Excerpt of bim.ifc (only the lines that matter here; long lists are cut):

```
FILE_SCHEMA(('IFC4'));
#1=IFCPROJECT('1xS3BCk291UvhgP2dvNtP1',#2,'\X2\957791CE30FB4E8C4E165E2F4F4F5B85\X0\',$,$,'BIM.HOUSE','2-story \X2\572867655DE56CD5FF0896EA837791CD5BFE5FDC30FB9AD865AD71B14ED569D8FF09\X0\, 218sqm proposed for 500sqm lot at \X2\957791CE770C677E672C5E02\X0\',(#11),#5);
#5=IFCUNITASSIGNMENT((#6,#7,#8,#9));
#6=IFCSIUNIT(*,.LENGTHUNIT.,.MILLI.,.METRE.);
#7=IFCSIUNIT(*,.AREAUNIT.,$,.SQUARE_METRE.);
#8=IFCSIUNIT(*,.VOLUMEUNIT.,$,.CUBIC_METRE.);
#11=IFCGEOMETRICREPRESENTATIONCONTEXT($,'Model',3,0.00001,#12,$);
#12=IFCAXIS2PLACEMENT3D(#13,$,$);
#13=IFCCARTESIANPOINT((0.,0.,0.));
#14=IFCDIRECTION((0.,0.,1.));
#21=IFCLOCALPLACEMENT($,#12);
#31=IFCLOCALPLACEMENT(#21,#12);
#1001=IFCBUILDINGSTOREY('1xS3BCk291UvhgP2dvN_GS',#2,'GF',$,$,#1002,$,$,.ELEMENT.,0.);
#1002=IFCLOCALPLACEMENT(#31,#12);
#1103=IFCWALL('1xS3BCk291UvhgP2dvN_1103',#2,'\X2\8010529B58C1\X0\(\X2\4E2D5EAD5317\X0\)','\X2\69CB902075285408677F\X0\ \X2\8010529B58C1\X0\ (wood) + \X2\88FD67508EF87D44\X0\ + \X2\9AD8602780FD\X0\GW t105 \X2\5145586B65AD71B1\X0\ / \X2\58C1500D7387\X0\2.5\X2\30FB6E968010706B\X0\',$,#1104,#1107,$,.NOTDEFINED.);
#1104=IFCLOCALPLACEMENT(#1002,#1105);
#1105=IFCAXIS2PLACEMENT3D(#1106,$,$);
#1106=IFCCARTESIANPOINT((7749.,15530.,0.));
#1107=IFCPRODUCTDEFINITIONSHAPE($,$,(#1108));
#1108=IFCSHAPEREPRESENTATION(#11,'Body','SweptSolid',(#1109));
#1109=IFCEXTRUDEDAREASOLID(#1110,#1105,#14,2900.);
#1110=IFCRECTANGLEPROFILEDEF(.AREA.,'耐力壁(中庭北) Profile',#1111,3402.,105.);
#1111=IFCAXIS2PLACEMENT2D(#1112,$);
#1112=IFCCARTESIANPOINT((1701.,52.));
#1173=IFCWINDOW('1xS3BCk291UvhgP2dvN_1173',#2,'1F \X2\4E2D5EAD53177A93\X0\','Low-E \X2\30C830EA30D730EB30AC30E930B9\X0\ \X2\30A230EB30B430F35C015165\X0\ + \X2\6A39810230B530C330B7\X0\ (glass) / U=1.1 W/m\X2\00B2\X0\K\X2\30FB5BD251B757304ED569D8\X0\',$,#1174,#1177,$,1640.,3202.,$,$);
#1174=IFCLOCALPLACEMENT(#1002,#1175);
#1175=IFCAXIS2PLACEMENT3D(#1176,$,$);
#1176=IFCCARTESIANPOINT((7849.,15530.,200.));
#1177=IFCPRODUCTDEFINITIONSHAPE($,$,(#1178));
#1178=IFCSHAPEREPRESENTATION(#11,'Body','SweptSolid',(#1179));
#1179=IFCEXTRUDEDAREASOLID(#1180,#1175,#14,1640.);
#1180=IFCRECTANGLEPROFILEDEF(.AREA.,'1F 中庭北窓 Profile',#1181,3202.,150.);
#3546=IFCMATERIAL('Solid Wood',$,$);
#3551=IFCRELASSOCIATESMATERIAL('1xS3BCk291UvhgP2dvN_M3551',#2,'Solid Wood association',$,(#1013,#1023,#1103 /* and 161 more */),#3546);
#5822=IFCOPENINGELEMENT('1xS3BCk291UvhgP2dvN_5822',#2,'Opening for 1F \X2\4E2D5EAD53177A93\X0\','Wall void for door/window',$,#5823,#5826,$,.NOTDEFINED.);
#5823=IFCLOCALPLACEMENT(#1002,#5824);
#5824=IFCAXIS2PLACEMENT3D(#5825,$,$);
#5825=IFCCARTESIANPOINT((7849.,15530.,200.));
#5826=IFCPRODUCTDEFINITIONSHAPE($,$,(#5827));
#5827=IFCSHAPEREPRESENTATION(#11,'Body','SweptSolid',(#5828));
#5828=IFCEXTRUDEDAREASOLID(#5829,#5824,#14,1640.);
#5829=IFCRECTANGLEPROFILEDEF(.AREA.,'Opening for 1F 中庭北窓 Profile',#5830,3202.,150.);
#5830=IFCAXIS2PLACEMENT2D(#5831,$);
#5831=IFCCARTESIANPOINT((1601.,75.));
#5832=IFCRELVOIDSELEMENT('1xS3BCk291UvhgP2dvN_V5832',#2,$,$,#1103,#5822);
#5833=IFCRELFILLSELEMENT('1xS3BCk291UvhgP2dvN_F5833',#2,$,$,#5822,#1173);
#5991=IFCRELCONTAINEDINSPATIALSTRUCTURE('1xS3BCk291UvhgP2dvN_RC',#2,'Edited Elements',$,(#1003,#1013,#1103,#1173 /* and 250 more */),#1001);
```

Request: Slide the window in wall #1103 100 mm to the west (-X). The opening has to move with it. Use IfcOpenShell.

```python
import ifcopenshell
import ifcopenshell.api.geometry
import ifcopenshell.util.placement
import ifcopenshell.util.unit

model = ifcopenshell.open("bim.ifc")
unit_scale = ifcopenshell.util.unit.calculate_unit_scale(model)

window = model.by_guid("1xS3BCk291UvhgP2dvN_1173")
opening = window.FillsVoids[0].RelatingOpeningElement
wall = opening.VoidsElements[0].RelatingBuildingElement

wall_matrix = ifcopenshell.util.placement.get_local_placement(wall.ObjectPlacement)
shift = wall_matrix[:3, 0] * -0.1 / unit_scale
before = ifcopenshell.util.placement.get_local_placement(window.ObjectPlacement)[:3, 3].copy()

# The window is not placed relative to its opening, so move both.
for product in (opening, window):
    matrix = ifcopenshell.util.placement.get_local_placement(product.ObjectPlacement)
    matrix[:3, 3] += shift
    ifcopenshell.api.geometry.edit_object_placement(model, product=product, matrix=matrix, is_si=False)

after = ifcopenshell.util.placement.get_local_placement(window.ObjectPlacement)[:3, 3]
print("window moved by", (after - before).round(3) + 0.0)

model.write("bim-out.ifc")
```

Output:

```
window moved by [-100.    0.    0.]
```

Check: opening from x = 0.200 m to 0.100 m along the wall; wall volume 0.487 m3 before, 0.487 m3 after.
